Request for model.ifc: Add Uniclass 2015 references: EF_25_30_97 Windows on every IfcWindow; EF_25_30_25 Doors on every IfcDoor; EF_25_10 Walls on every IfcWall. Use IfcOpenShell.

First a look at what the model holds.

```python
import ifcopenshell

model = ifcopenshell.open("model.ifc")
print(model.schema)
print("classifications:", [c.Name for c in model.by_type("IfcClassification")])
for ifc_class in ("IfcDoor", "IfcRoof", "IfcStair", "IfcWall", "IfcWindow"):
    print(ifc_class, len(model.by_type(ifc_class)))
```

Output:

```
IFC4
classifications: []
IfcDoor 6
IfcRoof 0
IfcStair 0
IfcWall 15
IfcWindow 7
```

```python
import ifcopenshell
import ifcopenshell.api.classification

model = ifcopenshell.open("model.ifc")

system = ifcopenshell.api.classification.add_classification(model, classification="Uniclass 2015")

codes = {
    "IfcWindow": ("EF_25_30_97", "Windows"),
    "IfcDoor": ("EF_25_30_25", "Doors"),
    "IfcWall": ("EF_25_10", "Walls"),
}
for ifc_class, (code, name) in codes.items():
    products = model.by_type(ifc_class)
    ifcopenshell.api.classification.add_reference(
        model, products=products, classification=system, identification=code, name=name
    )
    print(code, len(products))

model.write("model_v2.ifc")
```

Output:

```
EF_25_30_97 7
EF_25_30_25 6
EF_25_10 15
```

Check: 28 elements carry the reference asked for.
